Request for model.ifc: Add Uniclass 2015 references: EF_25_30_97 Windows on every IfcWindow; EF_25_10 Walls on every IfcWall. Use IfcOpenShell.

First a look at what the model holds.

```python
import ifcopenshell

model = ifcopenshell.open("model.ifc")
print(model.schema)
print("classifications:", [c.Name for c in model.by_type("IfcClassification")])
for ifc_class in ("IfcDoor", "IfcRoof", "IfcStair", "IfcWall", "IfcWindow"):
    print(ifc_class, len(model.by_type(ifc_class)))
```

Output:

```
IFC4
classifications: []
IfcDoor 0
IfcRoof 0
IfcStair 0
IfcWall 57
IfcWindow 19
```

```python
import ifcopenshell
import ifcopenshell.api.classification

model = ifcopenshell.open("model.ifc")

system = ifcopenshell.api.classification.add_classification(model, classification="Uniclass 2015")

codes = {
    "IfcWindow": ("EF_25_30_97", "Windows"),
    "IfcWall": ("EF_25_10", "Walls"),
}
for ifc_class, (code, name) in codes.items():
    products = model.by_type(ifc_class)
    ifcopenshell.api.classification.add_reference(
        model, products=products, classification=system, identification=code, name=name
    )
    print(code, len(products))

model.write("model_rev.ifc")
```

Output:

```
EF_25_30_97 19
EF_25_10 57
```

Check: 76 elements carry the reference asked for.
